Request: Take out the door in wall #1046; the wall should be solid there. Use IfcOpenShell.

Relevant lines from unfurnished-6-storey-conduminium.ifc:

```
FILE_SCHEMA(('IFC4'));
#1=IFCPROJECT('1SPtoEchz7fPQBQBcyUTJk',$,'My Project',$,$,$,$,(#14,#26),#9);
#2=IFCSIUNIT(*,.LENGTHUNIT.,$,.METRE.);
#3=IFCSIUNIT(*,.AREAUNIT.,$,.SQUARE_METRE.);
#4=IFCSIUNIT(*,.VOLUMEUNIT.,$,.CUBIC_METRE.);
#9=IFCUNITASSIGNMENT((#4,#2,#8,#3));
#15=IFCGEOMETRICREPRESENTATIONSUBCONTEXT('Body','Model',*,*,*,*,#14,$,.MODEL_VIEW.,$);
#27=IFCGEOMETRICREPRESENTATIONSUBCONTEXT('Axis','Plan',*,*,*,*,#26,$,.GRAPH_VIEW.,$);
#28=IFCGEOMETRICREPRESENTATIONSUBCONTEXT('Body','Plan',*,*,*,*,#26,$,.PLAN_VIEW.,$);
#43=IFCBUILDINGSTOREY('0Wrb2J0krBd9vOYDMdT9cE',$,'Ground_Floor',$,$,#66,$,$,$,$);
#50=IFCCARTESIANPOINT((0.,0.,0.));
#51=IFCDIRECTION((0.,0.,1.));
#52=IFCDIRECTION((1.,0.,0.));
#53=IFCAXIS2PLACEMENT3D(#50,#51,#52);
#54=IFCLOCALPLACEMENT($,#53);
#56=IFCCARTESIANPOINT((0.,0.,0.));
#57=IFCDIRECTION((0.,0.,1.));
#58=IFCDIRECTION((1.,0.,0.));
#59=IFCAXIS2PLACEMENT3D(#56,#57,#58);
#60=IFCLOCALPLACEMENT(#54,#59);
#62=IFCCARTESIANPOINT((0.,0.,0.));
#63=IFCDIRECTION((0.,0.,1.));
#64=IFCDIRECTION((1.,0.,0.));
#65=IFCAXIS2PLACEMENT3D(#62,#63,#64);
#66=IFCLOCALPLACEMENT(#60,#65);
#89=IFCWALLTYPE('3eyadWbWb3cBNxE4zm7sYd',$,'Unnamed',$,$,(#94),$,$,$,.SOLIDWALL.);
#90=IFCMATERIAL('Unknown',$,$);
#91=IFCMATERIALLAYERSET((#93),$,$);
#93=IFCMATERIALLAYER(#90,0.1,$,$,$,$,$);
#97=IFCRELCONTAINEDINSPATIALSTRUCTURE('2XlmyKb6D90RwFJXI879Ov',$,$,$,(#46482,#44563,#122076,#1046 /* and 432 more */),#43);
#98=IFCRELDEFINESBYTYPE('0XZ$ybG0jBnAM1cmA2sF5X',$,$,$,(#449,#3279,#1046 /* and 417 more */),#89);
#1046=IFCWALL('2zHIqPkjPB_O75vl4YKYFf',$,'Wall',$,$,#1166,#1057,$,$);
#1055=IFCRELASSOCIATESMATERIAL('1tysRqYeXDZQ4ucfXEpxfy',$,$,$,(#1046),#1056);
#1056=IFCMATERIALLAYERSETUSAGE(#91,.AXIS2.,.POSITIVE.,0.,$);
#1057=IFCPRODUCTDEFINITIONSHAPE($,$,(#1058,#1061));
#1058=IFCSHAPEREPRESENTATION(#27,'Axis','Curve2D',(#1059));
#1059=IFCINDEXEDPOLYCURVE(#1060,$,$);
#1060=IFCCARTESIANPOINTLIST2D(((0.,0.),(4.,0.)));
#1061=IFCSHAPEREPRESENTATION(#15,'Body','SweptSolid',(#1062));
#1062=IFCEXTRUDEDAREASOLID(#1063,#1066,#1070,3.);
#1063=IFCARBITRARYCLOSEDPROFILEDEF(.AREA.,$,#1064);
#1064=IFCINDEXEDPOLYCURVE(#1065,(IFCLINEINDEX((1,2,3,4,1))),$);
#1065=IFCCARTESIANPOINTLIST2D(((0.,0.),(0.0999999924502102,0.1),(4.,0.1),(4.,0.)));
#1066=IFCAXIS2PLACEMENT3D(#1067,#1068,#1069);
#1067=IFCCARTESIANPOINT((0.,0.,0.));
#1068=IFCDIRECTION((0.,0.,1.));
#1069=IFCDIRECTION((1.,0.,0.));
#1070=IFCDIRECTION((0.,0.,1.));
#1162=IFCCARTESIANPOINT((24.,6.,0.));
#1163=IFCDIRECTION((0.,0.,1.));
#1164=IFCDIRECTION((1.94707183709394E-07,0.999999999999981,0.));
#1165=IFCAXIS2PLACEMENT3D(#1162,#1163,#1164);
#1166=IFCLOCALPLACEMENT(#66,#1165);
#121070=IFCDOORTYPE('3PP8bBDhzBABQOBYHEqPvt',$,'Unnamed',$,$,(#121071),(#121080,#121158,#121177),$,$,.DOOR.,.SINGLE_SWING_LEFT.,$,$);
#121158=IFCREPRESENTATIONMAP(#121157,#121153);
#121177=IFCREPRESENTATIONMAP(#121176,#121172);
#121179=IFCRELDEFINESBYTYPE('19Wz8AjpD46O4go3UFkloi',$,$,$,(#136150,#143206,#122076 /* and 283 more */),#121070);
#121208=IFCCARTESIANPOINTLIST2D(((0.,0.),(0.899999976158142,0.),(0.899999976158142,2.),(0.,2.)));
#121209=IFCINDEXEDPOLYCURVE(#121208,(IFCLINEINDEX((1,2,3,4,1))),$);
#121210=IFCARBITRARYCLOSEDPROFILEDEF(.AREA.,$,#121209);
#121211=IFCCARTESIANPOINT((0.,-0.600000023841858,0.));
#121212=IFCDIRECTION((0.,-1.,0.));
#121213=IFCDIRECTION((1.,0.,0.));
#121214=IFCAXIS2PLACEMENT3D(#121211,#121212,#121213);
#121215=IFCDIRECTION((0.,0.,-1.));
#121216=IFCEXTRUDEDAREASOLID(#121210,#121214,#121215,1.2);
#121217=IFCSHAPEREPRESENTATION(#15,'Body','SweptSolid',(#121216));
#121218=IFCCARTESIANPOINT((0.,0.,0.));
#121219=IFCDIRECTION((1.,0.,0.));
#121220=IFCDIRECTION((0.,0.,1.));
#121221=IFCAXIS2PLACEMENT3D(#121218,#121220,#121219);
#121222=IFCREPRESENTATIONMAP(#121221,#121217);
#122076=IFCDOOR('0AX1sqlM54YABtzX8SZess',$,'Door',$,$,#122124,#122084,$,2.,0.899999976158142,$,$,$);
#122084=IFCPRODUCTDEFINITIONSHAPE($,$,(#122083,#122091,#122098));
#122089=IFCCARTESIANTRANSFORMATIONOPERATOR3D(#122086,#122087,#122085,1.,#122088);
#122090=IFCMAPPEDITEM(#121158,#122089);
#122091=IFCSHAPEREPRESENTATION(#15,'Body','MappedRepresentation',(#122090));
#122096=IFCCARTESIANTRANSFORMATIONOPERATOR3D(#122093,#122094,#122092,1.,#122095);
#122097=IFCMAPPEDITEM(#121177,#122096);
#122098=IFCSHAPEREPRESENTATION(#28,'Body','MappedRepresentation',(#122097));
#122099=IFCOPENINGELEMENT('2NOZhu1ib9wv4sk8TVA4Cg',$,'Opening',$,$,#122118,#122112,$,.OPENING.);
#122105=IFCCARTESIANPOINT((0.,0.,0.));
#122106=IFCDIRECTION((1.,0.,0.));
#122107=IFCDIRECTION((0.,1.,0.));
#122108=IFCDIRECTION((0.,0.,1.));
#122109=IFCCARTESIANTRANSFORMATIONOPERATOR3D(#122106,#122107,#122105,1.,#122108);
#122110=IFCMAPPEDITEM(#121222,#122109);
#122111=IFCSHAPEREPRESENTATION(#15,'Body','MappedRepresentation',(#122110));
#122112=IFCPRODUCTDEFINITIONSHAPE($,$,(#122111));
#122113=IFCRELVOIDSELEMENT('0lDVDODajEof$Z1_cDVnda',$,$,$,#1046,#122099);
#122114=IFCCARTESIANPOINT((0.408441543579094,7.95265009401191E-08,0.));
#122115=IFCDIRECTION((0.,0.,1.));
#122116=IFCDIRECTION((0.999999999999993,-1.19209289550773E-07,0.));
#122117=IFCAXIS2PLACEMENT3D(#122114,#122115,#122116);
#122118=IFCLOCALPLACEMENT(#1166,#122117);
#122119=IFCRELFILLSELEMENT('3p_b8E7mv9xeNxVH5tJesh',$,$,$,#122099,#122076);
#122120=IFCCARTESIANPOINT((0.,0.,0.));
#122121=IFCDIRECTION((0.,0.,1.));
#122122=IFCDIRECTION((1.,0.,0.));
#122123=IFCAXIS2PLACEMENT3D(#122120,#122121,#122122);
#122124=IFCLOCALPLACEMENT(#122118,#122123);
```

```python
import ifcopenshell
import ifcopenshell.api.feature
import ifcopenshell.api.root
import ifcopenshell.geom
import ifcopenshell.util.shape

model = ifcopenshell.open("unfurnished-6-storey-conduminium.ifc")
settings = ifcopenshell.geom.settings()


def volume(element):
    """Net volume in cubic metres, openings subtracted."""
    shape = ifcopenshell.geom.create_shape(settings, element)
    return ifcopenshell.util.shape.get_volume(shape.geometry)


door = model.by_guid("0AX1sqlM54YABtzX8SZess")
opening = door.FillsVoids[0].RelatingOpeningElement
wall = opening.VoidsElements[0].RelatingBuildingElement
before = volume(wall)

ifcopenshell.api.root.remove_product(model, product=door)
ifcopenshell.api.feature.remove_feature(model, feature=opening)

after = volume(wall)

print(f"wall volume {before:.3f} -> {after:.3f} m3")

model.write("unfurnished-6-storey-conduminium_v2.ifc")
```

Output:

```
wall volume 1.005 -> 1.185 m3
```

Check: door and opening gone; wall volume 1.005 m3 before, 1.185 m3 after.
